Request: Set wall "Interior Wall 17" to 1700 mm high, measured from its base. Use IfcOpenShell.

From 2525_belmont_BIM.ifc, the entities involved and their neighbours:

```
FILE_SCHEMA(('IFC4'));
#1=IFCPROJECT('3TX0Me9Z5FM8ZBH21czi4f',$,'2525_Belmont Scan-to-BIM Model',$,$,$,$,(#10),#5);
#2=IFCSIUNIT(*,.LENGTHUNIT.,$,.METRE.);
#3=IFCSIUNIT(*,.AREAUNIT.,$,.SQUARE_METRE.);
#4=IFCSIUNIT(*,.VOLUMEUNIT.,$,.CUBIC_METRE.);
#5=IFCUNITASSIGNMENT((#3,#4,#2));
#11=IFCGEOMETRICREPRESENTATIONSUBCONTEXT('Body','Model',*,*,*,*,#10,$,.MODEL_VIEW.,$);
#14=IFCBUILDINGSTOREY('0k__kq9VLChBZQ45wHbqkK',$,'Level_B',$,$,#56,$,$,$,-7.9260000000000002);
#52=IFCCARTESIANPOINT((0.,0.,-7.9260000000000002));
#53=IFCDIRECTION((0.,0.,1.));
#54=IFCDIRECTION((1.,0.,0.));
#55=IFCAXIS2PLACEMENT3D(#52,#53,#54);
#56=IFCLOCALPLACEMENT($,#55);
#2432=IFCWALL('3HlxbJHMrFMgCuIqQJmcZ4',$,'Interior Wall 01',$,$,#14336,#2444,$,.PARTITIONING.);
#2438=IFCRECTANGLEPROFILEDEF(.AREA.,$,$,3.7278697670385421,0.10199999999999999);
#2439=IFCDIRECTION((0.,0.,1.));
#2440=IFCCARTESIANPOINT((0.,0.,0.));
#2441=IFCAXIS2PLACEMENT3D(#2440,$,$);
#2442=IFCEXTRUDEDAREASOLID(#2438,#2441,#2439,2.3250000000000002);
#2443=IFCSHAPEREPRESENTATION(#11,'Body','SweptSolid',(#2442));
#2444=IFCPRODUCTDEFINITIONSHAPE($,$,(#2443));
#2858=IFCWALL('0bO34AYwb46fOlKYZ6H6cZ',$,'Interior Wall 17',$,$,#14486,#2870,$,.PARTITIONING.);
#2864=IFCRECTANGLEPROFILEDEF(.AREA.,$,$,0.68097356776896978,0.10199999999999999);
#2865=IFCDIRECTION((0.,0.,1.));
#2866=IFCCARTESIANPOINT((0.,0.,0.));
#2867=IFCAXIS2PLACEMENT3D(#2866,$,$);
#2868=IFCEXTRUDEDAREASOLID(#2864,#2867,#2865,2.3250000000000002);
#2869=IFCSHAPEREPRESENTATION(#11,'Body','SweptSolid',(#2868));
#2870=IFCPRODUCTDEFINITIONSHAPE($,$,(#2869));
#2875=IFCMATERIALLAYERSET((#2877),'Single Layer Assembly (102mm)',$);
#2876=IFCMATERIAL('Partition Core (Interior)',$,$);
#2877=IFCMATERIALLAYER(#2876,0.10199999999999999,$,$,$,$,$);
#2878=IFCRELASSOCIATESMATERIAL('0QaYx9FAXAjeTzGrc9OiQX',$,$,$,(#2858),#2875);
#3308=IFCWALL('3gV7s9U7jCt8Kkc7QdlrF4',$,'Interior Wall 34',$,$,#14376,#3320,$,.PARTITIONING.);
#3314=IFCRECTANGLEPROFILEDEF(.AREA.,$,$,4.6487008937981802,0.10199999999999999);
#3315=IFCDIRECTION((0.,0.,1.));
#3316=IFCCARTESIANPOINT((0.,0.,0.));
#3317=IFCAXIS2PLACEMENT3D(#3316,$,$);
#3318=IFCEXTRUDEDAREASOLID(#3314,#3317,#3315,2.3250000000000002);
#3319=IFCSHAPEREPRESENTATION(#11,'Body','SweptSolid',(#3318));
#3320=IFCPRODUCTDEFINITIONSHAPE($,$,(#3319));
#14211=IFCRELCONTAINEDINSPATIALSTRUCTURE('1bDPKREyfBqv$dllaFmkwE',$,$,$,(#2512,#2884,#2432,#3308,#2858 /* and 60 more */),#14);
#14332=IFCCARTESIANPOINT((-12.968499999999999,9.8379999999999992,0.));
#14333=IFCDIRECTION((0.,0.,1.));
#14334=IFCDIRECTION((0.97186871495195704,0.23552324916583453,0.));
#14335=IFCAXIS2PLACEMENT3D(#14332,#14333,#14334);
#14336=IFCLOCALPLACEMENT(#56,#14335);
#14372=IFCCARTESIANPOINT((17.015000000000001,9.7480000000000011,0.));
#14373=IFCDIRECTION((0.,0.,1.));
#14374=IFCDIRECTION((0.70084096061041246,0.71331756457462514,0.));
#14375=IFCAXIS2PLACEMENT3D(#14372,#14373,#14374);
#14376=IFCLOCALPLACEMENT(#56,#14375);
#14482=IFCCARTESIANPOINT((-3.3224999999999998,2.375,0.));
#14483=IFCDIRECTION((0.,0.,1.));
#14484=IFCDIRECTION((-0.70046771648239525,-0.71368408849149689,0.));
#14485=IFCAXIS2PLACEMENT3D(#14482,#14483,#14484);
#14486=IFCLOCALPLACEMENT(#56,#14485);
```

```python
import ifcopenshell
import ifcopenshell.geom
import ifcopenshell.util.representation
import ifcopenshell.util.shape
import ifcopenshell.util.unit

model = ifcopenshell.open("2525_belmont_BIM.ifc")
unit_scale = ifcopenshell.util.unit.calculate_unit_scale(model)
settings = ifcopenshell.geom.settings()


def volume(element):
    """Net volume in cubic metres, openings subtracted."""
    shape = ifcopenshell.geom.create_shape(settings, element)
    return ifcopenshell.util.shape.get_volume(shape.geometry)


wall = model.by_guid("0bO34AYwb46fOlKYZ6H6cZ")
before = volume(wall)

body = ifcopenshell.util.representation.get_representation(wall, "Model", "Body")
solid = body.Items[0]
old_height = solid.Depth
solid.Depth = 1.7 / unit_scale
after = volume(wall)

print(f"height {old_height:g} -> {solid.Depth:g}, volume {before:.3f} -> {after:.3f} m3")

model.write("2525_belmont_BIM_updated.ifc")
```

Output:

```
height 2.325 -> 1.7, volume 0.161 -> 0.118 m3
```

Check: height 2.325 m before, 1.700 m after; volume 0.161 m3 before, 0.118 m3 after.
